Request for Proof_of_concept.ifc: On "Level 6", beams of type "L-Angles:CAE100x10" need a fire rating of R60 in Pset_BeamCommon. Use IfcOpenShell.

First a look at what the model holds.

```python
import ifcopenshell
import ifcopenshell.util.element

model = ifcopenshell.open("Proof_of_concept.ifc")
print(model.schema)
storey = next(s for s in model.by_type("IfcBuildingStorey") if s.Name == "Level 6")
beams = [e for e in ifcopenshell.util.element.get_decomposition(storey) if e.is_a("IfcBeam")]
seen = {}
for e in beams:
    element_type = ifcopenshell.util.element.get_type(e)
    key = (element_type.Name if element_type != e and element_type else None, ifcopenshell.util.element.get_pset(e, "Pset_BeamCommon", "FireRating"))
    seen[key] = seen.get(key, 0) + 1
for (name, value), count in sorted(seen.items(), key=str):
    print(count, "x", name, "|", value)
```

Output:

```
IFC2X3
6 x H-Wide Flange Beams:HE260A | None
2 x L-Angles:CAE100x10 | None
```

```python
import ifcopenshell
import ifcopenshell.api.pset
import ifcopenshell.util.element

model = ifcopenshell.open("Proof_of_concept.ifc")

storey = next(s for s in model.by_type("IfcBuildingStorey") if s.Name == "Level 6")
beams = [e for e in ifcopenshell.util.element.get_decomposition(storey) if e.is_a("IfcBeam")]

count = 0
for e in beams:
    element_type = ifcopenshell.util.element.get_type(e)
    if element_type in (None, e) or element_type.Name != "L-Angles:CAE100x10":
        continue
    # add_pset returns the element's existing set when there is one.
    pset = ifcopenshell.api.pset.add_pset(model, product=e, name="Pset_BeamCommon")
    ifcopenshell.api.pset.edit_pset(model, pset=pset, properties={"FireRating": "R60"})
    count += 1

print(count, "beams updated")

model.write("Proof_of_concept_edited.ifc")
```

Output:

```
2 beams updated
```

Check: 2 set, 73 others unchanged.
